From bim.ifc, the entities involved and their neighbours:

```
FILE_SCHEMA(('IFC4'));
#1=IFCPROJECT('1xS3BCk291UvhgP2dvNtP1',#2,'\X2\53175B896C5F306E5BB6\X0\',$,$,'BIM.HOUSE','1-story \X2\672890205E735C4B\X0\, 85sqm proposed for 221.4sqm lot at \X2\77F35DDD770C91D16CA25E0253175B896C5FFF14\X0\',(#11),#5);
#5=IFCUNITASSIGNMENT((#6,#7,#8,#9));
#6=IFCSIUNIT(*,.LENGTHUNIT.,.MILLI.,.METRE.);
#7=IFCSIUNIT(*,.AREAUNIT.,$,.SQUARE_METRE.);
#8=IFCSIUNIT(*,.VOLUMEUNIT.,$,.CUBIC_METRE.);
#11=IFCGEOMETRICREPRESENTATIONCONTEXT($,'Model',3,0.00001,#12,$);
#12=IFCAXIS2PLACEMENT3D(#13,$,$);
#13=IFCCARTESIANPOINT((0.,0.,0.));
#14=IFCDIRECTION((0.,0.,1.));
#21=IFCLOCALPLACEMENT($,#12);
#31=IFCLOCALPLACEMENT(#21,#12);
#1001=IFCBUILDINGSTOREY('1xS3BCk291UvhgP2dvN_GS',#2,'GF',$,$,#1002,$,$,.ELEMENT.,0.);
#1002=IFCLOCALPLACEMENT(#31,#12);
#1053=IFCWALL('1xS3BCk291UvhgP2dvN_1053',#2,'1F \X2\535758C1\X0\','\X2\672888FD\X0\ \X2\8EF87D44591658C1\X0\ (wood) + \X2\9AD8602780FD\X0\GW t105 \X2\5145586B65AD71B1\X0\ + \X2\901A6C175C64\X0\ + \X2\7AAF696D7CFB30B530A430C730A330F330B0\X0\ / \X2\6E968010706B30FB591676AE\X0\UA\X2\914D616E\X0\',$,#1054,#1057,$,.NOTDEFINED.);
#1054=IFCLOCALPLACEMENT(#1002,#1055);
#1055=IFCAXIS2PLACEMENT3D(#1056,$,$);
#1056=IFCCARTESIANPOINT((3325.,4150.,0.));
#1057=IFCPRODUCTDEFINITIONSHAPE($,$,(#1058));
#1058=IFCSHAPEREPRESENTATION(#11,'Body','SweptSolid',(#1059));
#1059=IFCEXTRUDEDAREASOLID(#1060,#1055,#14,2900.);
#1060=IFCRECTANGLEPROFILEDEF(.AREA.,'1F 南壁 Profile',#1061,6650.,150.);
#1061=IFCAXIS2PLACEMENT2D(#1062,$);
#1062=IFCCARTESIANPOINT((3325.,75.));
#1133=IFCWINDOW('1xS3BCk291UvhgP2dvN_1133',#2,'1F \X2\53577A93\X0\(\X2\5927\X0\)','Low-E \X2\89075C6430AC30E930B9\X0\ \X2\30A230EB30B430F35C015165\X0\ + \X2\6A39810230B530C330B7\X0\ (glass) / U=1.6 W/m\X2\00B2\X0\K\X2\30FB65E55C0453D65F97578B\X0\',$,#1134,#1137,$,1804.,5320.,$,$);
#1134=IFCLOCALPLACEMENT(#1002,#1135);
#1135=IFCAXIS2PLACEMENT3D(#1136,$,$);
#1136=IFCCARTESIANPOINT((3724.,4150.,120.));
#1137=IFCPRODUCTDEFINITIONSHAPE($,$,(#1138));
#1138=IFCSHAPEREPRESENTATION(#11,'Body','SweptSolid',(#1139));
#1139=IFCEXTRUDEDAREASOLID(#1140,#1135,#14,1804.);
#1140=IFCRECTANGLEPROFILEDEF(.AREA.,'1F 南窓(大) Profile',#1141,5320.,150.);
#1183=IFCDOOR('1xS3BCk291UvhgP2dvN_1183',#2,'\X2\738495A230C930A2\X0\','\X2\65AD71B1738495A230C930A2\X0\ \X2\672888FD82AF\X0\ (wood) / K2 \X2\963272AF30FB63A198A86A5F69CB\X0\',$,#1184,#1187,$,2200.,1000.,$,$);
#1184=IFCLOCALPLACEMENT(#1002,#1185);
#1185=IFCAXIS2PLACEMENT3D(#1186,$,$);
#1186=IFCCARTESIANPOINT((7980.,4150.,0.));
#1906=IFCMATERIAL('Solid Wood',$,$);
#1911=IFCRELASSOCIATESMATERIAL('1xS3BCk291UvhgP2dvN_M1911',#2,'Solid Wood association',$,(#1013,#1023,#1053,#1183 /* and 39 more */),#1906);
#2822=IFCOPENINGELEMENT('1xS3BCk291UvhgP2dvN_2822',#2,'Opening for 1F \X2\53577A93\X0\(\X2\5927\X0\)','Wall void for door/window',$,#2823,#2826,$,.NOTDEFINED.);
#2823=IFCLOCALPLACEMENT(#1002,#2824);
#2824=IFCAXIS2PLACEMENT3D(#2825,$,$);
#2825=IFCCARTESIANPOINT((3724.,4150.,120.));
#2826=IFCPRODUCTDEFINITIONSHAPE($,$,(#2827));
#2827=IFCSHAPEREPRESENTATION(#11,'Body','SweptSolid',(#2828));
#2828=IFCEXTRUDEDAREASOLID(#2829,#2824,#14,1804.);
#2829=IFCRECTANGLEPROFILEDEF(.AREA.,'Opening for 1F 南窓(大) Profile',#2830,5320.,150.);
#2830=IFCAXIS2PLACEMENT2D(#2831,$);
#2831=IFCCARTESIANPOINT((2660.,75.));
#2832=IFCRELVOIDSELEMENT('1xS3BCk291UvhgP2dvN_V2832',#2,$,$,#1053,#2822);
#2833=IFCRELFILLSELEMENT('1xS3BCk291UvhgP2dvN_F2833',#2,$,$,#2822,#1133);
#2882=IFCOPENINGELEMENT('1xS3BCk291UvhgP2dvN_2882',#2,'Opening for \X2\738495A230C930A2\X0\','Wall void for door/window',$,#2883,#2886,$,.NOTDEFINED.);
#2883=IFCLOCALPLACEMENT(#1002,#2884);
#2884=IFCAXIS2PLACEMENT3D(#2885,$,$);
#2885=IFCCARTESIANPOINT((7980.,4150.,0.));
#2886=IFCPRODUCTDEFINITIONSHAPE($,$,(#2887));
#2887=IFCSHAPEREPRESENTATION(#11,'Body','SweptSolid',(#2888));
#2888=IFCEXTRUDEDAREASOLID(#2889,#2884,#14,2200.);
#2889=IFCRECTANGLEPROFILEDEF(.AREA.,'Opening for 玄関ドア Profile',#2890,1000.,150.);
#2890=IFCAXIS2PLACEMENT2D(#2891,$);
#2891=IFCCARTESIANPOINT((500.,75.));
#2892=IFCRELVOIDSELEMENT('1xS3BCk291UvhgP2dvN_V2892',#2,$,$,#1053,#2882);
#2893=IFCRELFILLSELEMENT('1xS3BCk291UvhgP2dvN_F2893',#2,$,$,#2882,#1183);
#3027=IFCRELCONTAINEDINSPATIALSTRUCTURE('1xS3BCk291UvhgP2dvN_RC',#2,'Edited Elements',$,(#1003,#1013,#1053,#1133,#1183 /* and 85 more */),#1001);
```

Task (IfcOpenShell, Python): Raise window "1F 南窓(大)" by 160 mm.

```python
import numpy as np
import ifcopenshell
import ifcopenshell.api.geometry
import ifcopenshell.util.placement
import ifcopenshell.util.unit

model = ifcopenshell.open("bim.ifc")
unit_scale = ifcopenshell.util.unit.calculate_unit_scale(model)

window = model.by_guid("1xS3BCk291UvhgP2dvN_1133")
opening = window.FillsVoids[0].RelatingOpeningElement
dz = 0.16 / unit_scale

shift = np.array([0.0, 0.0, dz])
# The window is not placed relative to its opening, so move both.
for product in (opening, window):
    matrix = ifcopenshell.util.placement.get_local_placement(product.ObjectPlacement)
    matrix[:3, 3] += shift
    ifcopenshell.api.geometry.edit_object_placement(model, product=product, matrix=matrix, is_si=False)

print(f"moved by {dz * unit_scale:+.3f} m")

model.write("bim_rev.ifc")
```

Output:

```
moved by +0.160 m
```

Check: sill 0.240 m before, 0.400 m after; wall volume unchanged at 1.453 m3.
